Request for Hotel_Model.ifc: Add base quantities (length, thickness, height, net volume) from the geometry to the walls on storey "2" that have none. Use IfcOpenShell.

First a look at what the model holds.

```python
import ifcopenshell
import ifcopenshell.util.element
import ifcopenshell.util.unit

model = ifcopenshell.open("Hotel_Model.ifc")
print(model.schema)
for unit_type in ("LENGTHUNIT", "AREAUNIT", "VOLUMEUNIT"):
    print(unit_type, ifcopenshell.util.unit.calculate_unit_scale(model, unit_type))
storey = next(s for s in model.by_type("IfcBuildingStorey") if s.Name == "2")
walls = [e for e in ifcopenshell.util.element.get_decomposition(storey) if e.is_a("IfcWall")]
for e in sorted(walls, key=lambda e: e.id()):
    print(e.id(), e.is_a(), e.Name, list(ifcopenshell.util.element.get_psets(e, qtos_only=True)), sep=" | ")
```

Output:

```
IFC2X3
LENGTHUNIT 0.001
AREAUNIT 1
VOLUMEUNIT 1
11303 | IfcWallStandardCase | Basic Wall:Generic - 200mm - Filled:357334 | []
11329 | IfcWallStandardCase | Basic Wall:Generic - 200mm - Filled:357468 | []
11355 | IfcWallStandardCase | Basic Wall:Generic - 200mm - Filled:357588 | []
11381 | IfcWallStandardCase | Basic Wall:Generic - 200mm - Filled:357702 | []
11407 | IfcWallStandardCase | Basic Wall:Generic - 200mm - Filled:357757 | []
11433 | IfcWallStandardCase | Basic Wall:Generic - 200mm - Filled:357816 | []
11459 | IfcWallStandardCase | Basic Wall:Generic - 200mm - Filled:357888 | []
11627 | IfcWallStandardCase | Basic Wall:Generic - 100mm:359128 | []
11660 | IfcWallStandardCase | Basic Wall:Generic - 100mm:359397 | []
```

```python
import ifcopenshell
import ifcopenshell.api.pset
import ifcopenshell.geom
import ifcopenshell.util.element
import ifcopenshell.util.shape
import ifcopenshell.util.unit

model = ifcopenshell.open("Hotel_Model.ifc")
unit_scale = ifcopenshell.util.unit.calculate_unit_scale(model)
volume_scale = ifcopenshell.util.unit.calculate_unit_scale(model, "VOLUMEUNIT")
settings = ifcopenshell.geom.settings()

storey = next(s for s in model.by_type("IfcBuildingStorey") if s.Name == "2")
walls = [e for e in ifcopenshell.util.element.get_decomposition(storey) if e.is_a("IfcWall")]

for e in sorted(walls, key=lambda e: e.id()):
    if ifcopenshell.util.element.get_psets(e, qtos_only=True, should_inherit=False):
        continue
    # Geometry comes back in metres, in the element's own axes.
    shape = ifcopenshell.geom.create_shape(settings, e)
    values = {
        "Length": ifcopenshell.util.shape.get_x(shape.geometry) / unit_scale,
        "Width": ifcopenshell.util.shape.get_y(shape.geometry) / unit_scale,
        "Height": ifcopenshell.util.shape.get_z(shape.geometry) / unit_scale,
        "NetVolume": ifcopenshell.util.shape.get_volume(shape.geometry) / volume_scale,
    }
    qto = ifcopenshell.api.pset.add_qto(model, product=e, name="BaseQuantities")
    ifcopenshell.api.pset.edit_qto(model, qto=qto, properties=values)
    print(e.id(), {k: round(v, 3) for k, v in values.items()})

model.write("Hotel_Model_rev.ifc")
```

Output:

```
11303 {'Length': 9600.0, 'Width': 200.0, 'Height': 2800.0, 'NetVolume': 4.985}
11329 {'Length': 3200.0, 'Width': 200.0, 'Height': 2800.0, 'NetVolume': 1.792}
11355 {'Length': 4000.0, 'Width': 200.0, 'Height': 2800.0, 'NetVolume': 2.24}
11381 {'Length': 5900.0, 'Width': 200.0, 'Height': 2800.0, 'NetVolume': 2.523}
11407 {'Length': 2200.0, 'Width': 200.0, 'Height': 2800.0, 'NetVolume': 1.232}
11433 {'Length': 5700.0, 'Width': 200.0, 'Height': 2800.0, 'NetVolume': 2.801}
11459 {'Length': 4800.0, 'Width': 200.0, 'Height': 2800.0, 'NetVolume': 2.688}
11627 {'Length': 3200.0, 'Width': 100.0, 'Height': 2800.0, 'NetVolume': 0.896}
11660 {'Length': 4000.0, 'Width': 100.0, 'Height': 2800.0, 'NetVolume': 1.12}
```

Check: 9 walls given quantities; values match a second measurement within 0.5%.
